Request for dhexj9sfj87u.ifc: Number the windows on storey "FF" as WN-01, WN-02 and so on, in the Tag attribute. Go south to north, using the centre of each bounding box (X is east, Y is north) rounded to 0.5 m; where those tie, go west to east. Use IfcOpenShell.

First a look at what the model holds.

```python
import ifcopenshell
import ifcopenshell.util.element
import ifcopenshell.util.placement

model = ifcopenshell.open("dhexj9sfj87u.ifc")
print(model.schema)
storey = next(s for s in model.by_type("IfcBuildingStorey") if s.Name == "FF")
windows = [e for e in ifcopenshell.util.element.get_decomposition(storey) if e.is_a("IfcWindow")]
for e in sorted(windows, key=lambda e: e.id()):
    origin = ifcopenshell.util.placement.get_local_placement(e.ObjectPlacement)[:3, 3]
    print(e.id(), e.Tag, e.Name, origin.round(2) + 0.0, sep=" | ")
```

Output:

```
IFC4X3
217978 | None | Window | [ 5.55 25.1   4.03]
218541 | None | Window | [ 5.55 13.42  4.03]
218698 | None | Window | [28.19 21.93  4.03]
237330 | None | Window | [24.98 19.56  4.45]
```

```python
import ifcopenshell
import ifcopenshell.geom
import ifcopenshell.util.element
import ifcopenshell.util.shape

model = ifcopenshell.open("dhexj9sfj87u.ifc")
settings = ifcopenshell.geom.settings()
settings.set("use-world-coords", True)


def centre(element):
    shape = ifcopenshell.geom.create_shape(settings, element)
    return ifcopenshell.util.shape.get_bbox_centroid(shape.geometry)


storey = next(s for s in model.by_type("IfcBuildingStorey") if s.Name == "FF")
windows = [e for e in ifcopenshell.util.element.get_decomposition(storey) if e.is_a("IfcWindow")]

# Insertion points can sit at a corner or the storey origin, so sort by the geometry (in metres).
centres = {e: centre(e) for e in windows}
windows.sort(key=lambda e: (round(centres[e][1] / 0.5), centres[e][0]))

for i, e in enumerate(windows, start=1):
    number = f"WN-{i:02d}"
    e.Tag = number
    print(e.id(), number)

model.write("dhexj9sfj87u_v2.ifc")
```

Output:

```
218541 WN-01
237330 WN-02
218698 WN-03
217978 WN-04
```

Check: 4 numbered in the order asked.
